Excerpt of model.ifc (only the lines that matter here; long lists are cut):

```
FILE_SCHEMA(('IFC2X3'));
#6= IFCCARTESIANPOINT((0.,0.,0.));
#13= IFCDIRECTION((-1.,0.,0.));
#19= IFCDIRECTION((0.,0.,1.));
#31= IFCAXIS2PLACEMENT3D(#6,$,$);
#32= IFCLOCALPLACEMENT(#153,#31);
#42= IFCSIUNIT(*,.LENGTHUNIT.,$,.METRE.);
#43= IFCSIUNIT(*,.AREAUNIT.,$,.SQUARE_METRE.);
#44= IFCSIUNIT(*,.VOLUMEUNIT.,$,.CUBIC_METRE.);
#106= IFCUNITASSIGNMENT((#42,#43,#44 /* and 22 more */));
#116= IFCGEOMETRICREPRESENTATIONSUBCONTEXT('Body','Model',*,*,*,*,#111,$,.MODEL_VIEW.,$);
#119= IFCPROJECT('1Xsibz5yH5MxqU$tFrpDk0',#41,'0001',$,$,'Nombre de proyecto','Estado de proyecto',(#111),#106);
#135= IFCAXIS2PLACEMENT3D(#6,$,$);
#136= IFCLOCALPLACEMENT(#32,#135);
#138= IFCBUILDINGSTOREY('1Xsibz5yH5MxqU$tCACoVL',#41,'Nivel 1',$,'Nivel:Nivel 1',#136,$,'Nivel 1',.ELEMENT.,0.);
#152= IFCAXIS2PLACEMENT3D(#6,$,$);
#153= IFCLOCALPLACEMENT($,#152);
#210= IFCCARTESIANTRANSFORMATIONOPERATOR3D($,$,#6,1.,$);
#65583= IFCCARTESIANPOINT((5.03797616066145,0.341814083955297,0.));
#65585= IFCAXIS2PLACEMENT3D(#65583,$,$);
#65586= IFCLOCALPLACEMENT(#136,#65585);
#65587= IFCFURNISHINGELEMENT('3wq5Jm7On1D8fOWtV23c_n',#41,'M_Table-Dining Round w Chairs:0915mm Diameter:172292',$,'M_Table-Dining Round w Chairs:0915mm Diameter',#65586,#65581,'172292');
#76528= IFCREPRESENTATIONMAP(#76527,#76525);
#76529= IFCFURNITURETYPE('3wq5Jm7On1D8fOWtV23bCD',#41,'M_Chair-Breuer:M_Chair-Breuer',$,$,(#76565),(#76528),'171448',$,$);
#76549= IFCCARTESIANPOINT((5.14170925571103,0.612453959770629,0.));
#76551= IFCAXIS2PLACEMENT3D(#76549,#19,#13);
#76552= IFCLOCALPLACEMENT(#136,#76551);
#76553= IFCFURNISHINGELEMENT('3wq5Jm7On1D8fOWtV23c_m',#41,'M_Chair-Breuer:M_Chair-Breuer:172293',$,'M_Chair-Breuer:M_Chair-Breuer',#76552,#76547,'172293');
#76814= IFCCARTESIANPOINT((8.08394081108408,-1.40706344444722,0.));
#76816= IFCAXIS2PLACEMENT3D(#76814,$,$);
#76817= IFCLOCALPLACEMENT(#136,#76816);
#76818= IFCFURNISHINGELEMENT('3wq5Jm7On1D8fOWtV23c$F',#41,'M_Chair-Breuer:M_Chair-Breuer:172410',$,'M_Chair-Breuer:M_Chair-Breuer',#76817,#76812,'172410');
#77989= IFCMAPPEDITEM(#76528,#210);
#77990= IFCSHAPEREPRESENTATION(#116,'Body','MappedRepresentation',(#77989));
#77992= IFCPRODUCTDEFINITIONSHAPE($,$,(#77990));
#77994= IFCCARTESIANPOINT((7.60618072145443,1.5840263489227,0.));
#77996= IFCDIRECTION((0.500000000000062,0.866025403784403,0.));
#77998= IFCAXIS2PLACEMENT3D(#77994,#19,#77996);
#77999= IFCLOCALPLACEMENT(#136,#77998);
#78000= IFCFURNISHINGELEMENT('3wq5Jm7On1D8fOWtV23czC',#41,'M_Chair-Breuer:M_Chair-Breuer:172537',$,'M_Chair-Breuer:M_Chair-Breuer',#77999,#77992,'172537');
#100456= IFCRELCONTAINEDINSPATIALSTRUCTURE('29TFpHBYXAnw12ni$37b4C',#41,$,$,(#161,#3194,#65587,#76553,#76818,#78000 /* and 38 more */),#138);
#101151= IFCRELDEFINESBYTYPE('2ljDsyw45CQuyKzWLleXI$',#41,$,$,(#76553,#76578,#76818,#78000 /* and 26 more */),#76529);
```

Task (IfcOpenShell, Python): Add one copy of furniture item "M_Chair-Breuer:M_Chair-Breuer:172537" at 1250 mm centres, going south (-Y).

```python
import numpy as np
import ifcopenshell
import ifcopenshell.api.geometry
import ifcopenshell.api.root
import ifcopenshell.util.element
import ifcopenshell.util.placement

model = ifcopenshell.open("model.ifc")


def reuse_history(source, copy):
    """copy_class also copies each property set's owner history, people and application; keep the originals."""
    for rel in copy.IsDefinedBy:
        if rel.is_a("IfcRelDefinesByProperties") and (history := rel.RelatingPropertyDefinition.OwnerHistory):
            rel.RelatingPropertyDefinition.OwnerHistory = source.OwnerHistory
            ifcopenshell.util.element.remove_deep2(model, history)


source = model.by_guid("3wq5Jm7On1D8fOWtV23czC")
base = ifcopenshell.util.placement.get_local_placement(source.ObjectPlacement)
step = np.array([0.0, -1.0, 0.0]) * 1.25

for i in range(1, 2):
    copy = ifcopenshell.api.root.copy_class(model, product=source)
    copy.Representation = ifcopenshell.util.element.copy_deep(
        model, source.Representation, exclude=["IfcGeometricRepresentationContext", "IfcRepresentationMap"]
    )
    copy.Name = "M_Chair-Breuer:M_Chair-Breuer"
    copy.Tag = None
    reuse_history(source, copy)
    matrix = base.copy()
    matrix[:3, 3] += i * step
    print("added at", matrix[:3, 3].round(3) + 0.0)
    ifcopenshell.api.geometry.edit_object_placement(model, product=copy, matrix=matrix, is_si=False)

model.write("model_rev.ifc")
```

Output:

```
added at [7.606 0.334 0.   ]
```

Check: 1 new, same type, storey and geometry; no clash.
